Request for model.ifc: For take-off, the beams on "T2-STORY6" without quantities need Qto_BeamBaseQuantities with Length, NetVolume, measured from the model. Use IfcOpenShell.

First a look at what the model holds.

```python
import ifcopenshell
import ifcopenshell.util.element
import ifcopenshell.util.unit

model = ifcopenshell.open("model.ifc")
print(model.schema)
for unit_type in ("LENGTHUNIT", "AREAUNIT", "VOLUMEUNIT"):
    print(unit_type, ifcopenshell.util.unit.calculate_unit_scale(model, unit_type))
storey = next(s for s in model.by_type("IfcBuildingStorey") if s.Name == "T2-STORY6")
beams = [e for e in ifcopenshell.util.element.get_decomposition(storey) if e.is_a("IfcBeam")]
for e in sorted(beams, key=lambda e: e.id()):
    print(e.id(), e.is_a(), e.Name, list(ifcopenshell.util.element.get_psets(e, qtos_only=True)), sep=" | ")
```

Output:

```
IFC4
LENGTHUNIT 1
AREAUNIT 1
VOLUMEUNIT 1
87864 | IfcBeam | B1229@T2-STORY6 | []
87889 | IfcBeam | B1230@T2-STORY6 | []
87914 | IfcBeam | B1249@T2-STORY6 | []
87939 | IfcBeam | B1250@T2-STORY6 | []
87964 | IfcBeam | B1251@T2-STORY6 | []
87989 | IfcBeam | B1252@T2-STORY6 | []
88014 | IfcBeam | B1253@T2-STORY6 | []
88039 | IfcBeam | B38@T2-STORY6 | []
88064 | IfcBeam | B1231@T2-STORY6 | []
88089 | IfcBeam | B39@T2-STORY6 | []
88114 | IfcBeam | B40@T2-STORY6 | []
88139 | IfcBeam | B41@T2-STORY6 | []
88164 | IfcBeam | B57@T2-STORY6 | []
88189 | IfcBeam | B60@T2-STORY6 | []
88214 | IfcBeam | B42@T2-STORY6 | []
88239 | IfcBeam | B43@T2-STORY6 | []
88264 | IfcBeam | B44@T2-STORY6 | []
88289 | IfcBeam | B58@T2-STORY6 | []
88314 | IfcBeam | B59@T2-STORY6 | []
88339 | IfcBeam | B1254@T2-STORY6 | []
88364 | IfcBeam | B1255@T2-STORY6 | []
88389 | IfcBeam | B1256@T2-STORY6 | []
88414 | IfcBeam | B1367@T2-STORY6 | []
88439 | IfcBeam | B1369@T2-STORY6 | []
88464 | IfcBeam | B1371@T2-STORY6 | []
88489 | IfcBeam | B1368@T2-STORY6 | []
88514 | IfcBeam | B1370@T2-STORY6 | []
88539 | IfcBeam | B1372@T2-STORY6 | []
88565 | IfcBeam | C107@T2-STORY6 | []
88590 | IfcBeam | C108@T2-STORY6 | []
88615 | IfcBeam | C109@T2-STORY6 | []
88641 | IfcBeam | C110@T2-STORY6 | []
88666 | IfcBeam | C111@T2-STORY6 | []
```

```python
import ifcopenshell
import ifcopenshell.api.pset
import ifcopenshell.geom
import ifcopenshell.util.element
import ifcopenshell.util.shape
import ifcopenshell.util.unit

model = ifcopenshell.open("model.ifc")
unit_scale = ifcopenshell.util.unit.calculate_unit_scale(model)
volume_scale = ifcopenshell.util.unit.calculate_unit_scale(model, "VOLUMEUNIT")
settings = ifcopenshell.geom.settings()

storey = next(s for s in model.by_type("IfcBuildingStorey") if s.Name == "T2-STORY6")
beams = [e for e in ifcopenshell.util.element.get_decomposition(storey) if e.is_a("IfcBeam")]

for e in sorted(beams, key=lambda e: e.id()):
    if ifcopenshell.util.element.get_psets(e, qtos_only=True, should_inherit=False):
        continue
    # Geometry comes back in metres, in the element's own axes.
    shape = ifcopenshell.geom.create_shape(settings, e)
    values = {
        "Length": ifcopenshell.util.shape.get_max_xyz(shape.geometry) / unit_scale,
        "NetVolume": ifcopenshell.util.shape.get_volume(shape.geometry) / volume_scale,
    }
    qto = ifcopenshell.api.pset.add_qto(model, product=e, name="Qto_BeamBaseQuantities")
    ifcopenshell.api.pset.edit_qto(model, qto=qto, properties=values)
    print(e.id(), {k: round(v, 3) for k, v in values.items()})

model.write("model_rev.ifc")
```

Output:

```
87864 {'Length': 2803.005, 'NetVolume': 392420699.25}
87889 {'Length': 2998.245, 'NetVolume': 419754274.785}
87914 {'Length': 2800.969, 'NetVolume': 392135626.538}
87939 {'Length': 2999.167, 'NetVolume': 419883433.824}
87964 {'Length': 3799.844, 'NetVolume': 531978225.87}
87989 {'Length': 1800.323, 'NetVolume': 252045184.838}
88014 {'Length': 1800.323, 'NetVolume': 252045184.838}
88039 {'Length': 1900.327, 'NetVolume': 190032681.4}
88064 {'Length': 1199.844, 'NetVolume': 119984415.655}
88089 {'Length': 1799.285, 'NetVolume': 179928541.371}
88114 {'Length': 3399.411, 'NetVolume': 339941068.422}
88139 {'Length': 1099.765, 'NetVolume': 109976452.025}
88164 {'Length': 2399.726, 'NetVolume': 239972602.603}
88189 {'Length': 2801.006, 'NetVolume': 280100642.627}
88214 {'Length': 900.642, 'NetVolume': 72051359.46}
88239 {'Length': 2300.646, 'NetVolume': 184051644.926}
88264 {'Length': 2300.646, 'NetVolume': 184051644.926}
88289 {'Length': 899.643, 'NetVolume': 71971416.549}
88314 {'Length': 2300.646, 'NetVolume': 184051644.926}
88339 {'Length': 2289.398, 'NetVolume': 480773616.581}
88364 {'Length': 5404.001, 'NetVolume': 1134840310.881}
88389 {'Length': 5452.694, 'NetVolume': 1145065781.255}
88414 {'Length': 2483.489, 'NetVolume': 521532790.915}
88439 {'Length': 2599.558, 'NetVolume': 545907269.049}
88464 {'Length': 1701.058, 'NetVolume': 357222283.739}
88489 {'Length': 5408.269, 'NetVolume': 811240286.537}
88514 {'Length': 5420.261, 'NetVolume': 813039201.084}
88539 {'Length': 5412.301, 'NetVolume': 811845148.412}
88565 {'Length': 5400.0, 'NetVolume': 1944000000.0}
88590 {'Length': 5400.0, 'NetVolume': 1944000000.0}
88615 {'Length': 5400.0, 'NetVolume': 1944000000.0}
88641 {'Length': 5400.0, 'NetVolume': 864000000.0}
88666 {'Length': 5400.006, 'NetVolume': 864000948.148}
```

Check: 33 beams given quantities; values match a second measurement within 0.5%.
